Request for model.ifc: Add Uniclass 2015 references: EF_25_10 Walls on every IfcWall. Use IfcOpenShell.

First a look at what the model holds.

```python
import ifcopenshell

model = ifcopenshell.open("model.ifc")
print(model.schema)
print("classifications:", [c.Name for c in model.by_type("IfcClassification")])
for ifc_class in ("IfcDoor", "IfcRoof", "IfcStair", "IfcWall", "IfcWindow"):
    print(ifc_class, len(model.by_type(ifc_class)))
```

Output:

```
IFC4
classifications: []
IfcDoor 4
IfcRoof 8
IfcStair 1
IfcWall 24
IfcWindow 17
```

```python
import ifcopenshell
import ifcopenshell.api.classification

model = ifcopenshell.open("model.ifc")

system = ifcopenshell.api.classification.add_classification(model, classification="Uniclass 2015")

codes = {
    "IfcWall": ("EF_25_10", "Walls"),
}
for ifc_class, (code, name) in codes.items():
    products = model.by_type(ifc_class)
    ifcopenshell.api.classification.add_reference(
        model, products=products, classification=system, identification=code, name=name
    )
    print(code, len(products))

model.write("model_v2.ifc")
```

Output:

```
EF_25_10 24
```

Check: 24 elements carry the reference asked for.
